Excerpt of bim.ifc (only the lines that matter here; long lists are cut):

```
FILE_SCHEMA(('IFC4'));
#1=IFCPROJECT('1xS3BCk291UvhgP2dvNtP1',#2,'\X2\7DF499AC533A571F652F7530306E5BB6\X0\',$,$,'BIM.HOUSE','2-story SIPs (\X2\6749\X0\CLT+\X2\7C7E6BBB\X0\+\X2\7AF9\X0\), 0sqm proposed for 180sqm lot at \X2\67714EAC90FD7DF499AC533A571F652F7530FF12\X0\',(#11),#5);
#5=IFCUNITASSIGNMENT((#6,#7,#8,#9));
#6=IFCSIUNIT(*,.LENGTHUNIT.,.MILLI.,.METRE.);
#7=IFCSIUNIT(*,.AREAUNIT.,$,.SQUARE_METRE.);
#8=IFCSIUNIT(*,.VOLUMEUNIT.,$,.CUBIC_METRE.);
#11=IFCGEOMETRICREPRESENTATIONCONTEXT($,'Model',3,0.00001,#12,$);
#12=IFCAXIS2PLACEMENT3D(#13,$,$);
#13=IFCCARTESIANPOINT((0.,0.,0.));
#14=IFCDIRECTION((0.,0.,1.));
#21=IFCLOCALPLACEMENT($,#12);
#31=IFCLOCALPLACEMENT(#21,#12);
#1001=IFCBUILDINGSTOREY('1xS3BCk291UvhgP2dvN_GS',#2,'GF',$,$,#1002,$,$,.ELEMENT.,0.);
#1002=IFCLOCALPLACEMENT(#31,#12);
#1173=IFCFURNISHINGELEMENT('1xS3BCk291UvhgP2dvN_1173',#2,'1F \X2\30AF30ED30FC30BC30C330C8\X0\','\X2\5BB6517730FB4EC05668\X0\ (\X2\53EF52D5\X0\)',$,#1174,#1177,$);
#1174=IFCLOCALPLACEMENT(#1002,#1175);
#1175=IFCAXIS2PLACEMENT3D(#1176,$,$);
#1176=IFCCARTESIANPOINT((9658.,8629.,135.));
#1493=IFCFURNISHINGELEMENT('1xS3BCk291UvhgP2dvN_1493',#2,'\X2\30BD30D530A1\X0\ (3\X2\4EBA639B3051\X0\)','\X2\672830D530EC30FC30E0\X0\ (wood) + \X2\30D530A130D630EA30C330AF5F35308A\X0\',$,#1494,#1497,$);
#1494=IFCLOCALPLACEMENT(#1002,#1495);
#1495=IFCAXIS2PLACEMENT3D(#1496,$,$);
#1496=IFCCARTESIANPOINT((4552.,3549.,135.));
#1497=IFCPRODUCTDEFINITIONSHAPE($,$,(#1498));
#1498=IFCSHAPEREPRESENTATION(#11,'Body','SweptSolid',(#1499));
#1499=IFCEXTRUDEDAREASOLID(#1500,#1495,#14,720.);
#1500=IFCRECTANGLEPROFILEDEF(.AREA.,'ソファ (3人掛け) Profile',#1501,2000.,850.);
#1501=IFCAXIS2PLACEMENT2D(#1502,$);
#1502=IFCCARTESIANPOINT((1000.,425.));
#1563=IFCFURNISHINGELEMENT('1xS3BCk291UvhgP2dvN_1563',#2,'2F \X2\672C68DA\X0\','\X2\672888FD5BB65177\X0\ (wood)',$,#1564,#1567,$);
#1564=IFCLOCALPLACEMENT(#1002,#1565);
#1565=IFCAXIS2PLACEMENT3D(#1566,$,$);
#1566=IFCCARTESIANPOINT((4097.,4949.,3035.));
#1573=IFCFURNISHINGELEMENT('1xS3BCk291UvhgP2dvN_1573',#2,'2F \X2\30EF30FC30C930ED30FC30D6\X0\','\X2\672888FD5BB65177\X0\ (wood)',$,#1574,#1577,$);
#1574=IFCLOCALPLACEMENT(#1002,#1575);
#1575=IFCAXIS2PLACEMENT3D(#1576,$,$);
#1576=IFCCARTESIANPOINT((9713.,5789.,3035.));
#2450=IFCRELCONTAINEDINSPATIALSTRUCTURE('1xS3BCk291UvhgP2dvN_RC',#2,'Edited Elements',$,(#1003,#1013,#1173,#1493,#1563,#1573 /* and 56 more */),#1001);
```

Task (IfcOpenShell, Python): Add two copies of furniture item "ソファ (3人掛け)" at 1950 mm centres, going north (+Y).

```python
import numpy as np
import ifcopenshell
import ifcopenshell.api.geometry
import ifcopenshell.api.root
import ifcopenshell.util.element
import ifcopenshell.util.placement
import ifcopenshell.util.unit

model = ifcopenshell.open("bim.ifc")
unit_scale = ifcopenshell.util.unit.calculate_unit_scale(model)


def reuse_history(source, copy):
    """copy_class also copies each property set's owner history, people and application; keep the originals."""
    for rel in copy.IsDefinedBy:
        if rel.is_a("IfcRelDefinesByProperties") and (history := rel.RelatingPropertyDefinition.OwnerHistory):
            rel.RelatingPropertyDefinition.OwnerHistory = source.OwnerHistory
            ifcopenshell.util.element.remove_deep2(model, history)


source = model.by_guid("1xS3BCk291UvhgP2dvN_1493")
base = ifcopenshell.util.placement.get_local_placement(source.ObjectPlacement)
step = np.array([0.0, 1.0, 0.0]) * 1.95 / unit_scale

for i in range(1, 3):
    copy = ifcopenshell.api.root.copy_class(model, product=source)
    copy.Representation = ifcopenshell.util.element.copy_deep(
        model, source.Representation, exclude=["IfcGeometricRepresentationContext", "IfcRepresentationMap"]
    )
    reuse_history(source, copy)
    matrix = base.copy()
    matrix[:3, 3] += i * step
    print("added at", matrix[:3, 3].round(3) + 0.0)
    ifcopenshell.api.geometry.edit_object_placement(model, product=copy, matrix=matrix, is_si=False)

model.write("bim_updated.ifc")
```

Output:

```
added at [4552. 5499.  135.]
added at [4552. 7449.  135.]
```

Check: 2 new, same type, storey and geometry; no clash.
